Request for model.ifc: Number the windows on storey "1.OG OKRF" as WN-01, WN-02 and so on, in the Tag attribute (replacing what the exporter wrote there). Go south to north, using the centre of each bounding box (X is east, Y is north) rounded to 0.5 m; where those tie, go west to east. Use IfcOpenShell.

First a look at what the model holds.

```python
import ifcopenshell
import ifcopenshell.util.element
import ifcopenshell.util.placement

model = ifcopenshell.open("model.ifc")
print(model.schema)
storey = next(s for s in model.by_type("IfcBuildingStorey") if s.Name == "1.OG OKRF")
windows = [e for e in ifcopenshell.util.element.get_decomposition(storey) if e.is_a("IfcWindow")]
for e in sorted(windows, key=lambda e: e.id()):
    origin = ifcopenshell.util.placement.get_local_placement(e.ObjectPlacement)[:3, 3]
    print(e.id(), e.Tag, e.Name, origin.round(2) + 0.0, sep=" | ")
```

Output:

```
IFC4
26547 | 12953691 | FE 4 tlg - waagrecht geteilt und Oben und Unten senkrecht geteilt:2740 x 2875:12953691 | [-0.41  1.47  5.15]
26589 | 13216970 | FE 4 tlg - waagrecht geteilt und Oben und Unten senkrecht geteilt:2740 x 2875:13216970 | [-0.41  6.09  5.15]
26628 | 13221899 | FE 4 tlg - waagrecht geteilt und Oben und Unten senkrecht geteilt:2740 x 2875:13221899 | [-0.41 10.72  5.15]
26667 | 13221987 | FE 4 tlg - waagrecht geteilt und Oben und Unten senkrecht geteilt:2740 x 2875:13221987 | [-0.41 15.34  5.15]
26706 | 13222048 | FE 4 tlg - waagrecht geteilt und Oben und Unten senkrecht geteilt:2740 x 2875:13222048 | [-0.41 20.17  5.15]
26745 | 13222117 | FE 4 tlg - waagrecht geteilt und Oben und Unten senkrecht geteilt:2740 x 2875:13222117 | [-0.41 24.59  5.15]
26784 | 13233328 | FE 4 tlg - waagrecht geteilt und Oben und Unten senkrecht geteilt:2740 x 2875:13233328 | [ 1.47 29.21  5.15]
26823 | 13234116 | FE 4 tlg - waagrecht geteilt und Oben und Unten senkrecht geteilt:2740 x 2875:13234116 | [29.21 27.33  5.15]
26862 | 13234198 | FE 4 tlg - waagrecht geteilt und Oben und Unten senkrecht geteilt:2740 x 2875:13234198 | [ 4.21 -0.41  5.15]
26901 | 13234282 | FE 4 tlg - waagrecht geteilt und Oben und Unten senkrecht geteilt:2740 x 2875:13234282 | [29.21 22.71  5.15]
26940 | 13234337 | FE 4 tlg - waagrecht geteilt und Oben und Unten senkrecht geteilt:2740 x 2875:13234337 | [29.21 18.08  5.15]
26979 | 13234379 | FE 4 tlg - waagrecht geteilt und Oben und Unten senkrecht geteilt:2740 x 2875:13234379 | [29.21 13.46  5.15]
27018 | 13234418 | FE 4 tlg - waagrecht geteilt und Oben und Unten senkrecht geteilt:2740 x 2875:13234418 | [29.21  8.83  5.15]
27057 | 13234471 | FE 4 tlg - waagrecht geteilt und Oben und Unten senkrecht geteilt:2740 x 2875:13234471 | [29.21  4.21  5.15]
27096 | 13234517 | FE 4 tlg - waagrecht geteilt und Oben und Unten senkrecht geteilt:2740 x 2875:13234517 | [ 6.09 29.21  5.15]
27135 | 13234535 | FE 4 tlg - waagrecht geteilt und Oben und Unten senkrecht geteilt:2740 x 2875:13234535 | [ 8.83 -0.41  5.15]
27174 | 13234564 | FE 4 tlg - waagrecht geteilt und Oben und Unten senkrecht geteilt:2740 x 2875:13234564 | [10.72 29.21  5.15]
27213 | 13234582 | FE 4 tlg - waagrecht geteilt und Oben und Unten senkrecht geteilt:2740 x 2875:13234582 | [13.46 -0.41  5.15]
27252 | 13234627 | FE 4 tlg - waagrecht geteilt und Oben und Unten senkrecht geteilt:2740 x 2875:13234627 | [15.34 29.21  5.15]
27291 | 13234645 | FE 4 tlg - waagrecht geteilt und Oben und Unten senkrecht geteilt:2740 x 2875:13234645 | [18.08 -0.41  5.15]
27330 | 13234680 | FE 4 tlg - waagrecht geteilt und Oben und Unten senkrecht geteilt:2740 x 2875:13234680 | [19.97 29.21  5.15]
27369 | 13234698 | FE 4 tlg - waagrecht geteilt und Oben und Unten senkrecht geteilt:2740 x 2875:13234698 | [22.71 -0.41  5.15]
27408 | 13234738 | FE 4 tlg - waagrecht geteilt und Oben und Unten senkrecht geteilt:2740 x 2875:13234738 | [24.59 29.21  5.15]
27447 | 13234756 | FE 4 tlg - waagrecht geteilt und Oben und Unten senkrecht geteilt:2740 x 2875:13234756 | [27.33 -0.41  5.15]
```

```python
import ifcopenshell
import ifcopenshell.geom
import ifcopenshell.util.element
import ifcopenshell.util.shape

model = ifcopenshell.open("model.ifc")
settings = ifcopenshell.geom.settings()
settings.set("use-world-coords", True)


def centre(element):
    shape = ifcopenshell.geom.create_shape(settings, element)
    return ifcopenshell.util.shape.get_bbox_centroid(shape.geometry)


storey = next(s for s in model.by_type("IfcBuildingStorey") if s.Name == "1.OG OKRF")
windows = [e for e in ifcopenshell.util.element.get_decomposition(storey) if e.is_a("IfcWindow")]

# Insertion points can sit at a corner or the storey origin, so sort by the geometry (in metres).
centres = {e: centre(e) for e in windows}
windows.sort(key=lambda e: (round(centres[e][1] / 0.5), centres[e][0]))

for i, e in enumerate(windows, start=1):
    number = f"WN-{i:02d}"
    e.Tag = number
    print(e.id(), number)

model.write("model_v2.ifc")
```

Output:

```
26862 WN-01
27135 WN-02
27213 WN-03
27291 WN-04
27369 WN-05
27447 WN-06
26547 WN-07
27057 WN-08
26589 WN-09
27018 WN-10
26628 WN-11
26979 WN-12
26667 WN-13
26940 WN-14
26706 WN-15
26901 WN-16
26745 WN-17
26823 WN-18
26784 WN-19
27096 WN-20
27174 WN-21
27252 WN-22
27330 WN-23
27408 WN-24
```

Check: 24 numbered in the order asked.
